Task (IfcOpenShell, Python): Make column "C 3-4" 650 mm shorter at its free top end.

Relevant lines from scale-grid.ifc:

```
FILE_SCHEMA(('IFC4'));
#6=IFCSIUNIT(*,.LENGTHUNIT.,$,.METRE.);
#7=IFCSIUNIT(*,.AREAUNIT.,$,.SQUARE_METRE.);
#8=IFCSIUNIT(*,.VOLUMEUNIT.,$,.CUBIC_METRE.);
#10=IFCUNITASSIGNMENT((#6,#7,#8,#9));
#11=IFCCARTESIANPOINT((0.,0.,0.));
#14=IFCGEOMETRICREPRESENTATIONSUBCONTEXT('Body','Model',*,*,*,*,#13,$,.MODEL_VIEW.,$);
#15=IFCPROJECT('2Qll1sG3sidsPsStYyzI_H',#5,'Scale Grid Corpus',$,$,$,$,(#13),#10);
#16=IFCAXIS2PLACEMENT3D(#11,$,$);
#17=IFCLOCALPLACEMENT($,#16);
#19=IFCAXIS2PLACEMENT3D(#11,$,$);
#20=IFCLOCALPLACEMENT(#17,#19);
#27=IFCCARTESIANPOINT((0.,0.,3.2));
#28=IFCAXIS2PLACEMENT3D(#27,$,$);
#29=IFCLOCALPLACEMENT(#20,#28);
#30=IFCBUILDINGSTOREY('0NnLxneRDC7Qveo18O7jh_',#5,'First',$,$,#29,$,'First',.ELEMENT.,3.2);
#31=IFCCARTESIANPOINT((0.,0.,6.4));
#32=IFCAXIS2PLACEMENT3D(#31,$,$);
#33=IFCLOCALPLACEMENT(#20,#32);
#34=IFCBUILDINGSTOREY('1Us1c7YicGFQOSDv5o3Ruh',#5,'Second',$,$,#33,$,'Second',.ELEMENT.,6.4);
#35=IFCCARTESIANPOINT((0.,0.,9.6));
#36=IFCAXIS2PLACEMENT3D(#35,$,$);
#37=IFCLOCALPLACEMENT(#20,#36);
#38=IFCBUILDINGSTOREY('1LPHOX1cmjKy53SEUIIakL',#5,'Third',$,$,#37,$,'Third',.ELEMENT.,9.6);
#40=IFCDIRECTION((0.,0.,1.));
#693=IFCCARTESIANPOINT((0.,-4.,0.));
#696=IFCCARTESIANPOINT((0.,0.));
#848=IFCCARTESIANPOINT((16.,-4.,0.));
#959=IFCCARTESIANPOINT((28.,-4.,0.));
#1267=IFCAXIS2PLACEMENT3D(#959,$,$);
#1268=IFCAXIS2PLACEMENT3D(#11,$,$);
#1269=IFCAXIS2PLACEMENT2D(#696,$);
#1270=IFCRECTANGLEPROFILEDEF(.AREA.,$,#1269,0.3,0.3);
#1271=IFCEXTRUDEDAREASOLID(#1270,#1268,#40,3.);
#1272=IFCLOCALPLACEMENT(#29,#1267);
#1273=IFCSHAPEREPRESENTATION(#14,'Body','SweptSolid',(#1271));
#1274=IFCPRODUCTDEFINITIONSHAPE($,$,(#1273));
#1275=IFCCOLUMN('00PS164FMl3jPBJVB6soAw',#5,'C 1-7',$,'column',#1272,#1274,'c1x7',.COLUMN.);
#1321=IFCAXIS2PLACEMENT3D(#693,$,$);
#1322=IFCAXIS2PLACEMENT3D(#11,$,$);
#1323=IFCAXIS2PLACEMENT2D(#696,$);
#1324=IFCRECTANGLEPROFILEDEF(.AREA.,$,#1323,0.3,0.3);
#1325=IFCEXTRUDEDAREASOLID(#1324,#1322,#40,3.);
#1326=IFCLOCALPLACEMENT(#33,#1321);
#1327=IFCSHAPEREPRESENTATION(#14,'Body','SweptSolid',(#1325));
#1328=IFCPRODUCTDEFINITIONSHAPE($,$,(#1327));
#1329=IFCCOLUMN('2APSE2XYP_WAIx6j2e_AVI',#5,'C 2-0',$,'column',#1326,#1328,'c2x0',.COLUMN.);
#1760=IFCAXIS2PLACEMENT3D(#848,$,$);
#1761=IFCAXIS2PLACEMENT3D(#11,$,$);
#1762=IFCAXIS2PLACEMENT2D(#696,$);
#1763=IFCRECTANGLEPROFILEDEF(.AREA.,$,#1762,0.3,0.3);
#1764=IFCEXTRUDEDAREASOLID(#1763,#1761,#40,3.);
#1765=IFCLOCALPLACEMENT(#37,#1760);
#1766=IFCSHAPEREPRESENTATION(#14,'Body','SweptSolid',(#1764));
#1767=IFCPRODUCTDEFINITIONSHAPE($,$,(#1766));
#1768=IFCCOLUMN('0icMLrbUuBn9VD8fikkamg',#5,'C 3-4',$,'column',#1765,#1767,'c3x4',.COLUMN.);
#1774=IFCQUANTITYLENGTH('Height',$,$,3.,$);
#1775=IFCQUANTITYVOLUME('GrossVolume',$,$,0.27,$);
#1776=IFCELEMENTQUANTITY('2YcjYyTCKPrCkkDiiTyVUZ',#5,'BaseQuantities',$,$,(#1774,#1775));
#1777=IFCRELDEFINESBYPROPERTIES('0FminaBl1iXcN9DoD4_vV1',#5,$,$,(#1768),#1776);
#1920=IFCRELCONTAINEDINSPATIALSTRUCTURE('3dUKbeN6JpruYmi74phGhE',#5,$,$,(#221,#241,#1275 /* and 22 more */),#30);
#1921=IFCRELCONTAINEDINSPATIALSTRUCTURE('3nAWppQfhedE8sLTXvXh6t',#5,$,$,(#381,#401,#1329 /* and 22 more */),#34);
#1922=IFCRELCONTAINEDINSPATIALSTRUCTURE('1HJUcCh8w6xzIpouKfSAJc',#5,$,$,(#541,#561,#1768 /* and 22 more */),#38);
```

```python
import ifcopenshell
import ifcopenshell.api.pset
import ifcopenshell.util.element
import ifcopenshell.util.representation

model = ifcopenshell.open("scale-grid.ifc")

member = model.by_guid("0icMLrbUuBn9VD8fikkamg")
change = -0.65

# The extrusion runs towards the end named, so only its depth changes.
body = ifcopenshell.util.representation.get_representation(member, "Model", "Body")
solid = body.Items[0]
old_length = solid.Depth
solid.Depth += change

# Update the stored length and volume.
qto = model.by_id(ifcopenshell.util.element.get_pset(member, "BaseQuantities", should_inherit=False)["id"])
ifcopenshell.api.pset.edit_qto(model, qto=qto, properties={
    "Height": solid.Depth,
    "GrossVolume": ifcopenshell.util.element.get_pset(member, "BaseQuantities", "GrossVolume") * solid.Depth / old_length,
})

print(f"length {old_length:g} -> {solid.Depth:g}")

model.write("scale-grid_edited.ifc")
```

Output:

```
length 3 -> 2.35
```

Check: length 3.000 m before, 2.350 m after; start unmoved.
